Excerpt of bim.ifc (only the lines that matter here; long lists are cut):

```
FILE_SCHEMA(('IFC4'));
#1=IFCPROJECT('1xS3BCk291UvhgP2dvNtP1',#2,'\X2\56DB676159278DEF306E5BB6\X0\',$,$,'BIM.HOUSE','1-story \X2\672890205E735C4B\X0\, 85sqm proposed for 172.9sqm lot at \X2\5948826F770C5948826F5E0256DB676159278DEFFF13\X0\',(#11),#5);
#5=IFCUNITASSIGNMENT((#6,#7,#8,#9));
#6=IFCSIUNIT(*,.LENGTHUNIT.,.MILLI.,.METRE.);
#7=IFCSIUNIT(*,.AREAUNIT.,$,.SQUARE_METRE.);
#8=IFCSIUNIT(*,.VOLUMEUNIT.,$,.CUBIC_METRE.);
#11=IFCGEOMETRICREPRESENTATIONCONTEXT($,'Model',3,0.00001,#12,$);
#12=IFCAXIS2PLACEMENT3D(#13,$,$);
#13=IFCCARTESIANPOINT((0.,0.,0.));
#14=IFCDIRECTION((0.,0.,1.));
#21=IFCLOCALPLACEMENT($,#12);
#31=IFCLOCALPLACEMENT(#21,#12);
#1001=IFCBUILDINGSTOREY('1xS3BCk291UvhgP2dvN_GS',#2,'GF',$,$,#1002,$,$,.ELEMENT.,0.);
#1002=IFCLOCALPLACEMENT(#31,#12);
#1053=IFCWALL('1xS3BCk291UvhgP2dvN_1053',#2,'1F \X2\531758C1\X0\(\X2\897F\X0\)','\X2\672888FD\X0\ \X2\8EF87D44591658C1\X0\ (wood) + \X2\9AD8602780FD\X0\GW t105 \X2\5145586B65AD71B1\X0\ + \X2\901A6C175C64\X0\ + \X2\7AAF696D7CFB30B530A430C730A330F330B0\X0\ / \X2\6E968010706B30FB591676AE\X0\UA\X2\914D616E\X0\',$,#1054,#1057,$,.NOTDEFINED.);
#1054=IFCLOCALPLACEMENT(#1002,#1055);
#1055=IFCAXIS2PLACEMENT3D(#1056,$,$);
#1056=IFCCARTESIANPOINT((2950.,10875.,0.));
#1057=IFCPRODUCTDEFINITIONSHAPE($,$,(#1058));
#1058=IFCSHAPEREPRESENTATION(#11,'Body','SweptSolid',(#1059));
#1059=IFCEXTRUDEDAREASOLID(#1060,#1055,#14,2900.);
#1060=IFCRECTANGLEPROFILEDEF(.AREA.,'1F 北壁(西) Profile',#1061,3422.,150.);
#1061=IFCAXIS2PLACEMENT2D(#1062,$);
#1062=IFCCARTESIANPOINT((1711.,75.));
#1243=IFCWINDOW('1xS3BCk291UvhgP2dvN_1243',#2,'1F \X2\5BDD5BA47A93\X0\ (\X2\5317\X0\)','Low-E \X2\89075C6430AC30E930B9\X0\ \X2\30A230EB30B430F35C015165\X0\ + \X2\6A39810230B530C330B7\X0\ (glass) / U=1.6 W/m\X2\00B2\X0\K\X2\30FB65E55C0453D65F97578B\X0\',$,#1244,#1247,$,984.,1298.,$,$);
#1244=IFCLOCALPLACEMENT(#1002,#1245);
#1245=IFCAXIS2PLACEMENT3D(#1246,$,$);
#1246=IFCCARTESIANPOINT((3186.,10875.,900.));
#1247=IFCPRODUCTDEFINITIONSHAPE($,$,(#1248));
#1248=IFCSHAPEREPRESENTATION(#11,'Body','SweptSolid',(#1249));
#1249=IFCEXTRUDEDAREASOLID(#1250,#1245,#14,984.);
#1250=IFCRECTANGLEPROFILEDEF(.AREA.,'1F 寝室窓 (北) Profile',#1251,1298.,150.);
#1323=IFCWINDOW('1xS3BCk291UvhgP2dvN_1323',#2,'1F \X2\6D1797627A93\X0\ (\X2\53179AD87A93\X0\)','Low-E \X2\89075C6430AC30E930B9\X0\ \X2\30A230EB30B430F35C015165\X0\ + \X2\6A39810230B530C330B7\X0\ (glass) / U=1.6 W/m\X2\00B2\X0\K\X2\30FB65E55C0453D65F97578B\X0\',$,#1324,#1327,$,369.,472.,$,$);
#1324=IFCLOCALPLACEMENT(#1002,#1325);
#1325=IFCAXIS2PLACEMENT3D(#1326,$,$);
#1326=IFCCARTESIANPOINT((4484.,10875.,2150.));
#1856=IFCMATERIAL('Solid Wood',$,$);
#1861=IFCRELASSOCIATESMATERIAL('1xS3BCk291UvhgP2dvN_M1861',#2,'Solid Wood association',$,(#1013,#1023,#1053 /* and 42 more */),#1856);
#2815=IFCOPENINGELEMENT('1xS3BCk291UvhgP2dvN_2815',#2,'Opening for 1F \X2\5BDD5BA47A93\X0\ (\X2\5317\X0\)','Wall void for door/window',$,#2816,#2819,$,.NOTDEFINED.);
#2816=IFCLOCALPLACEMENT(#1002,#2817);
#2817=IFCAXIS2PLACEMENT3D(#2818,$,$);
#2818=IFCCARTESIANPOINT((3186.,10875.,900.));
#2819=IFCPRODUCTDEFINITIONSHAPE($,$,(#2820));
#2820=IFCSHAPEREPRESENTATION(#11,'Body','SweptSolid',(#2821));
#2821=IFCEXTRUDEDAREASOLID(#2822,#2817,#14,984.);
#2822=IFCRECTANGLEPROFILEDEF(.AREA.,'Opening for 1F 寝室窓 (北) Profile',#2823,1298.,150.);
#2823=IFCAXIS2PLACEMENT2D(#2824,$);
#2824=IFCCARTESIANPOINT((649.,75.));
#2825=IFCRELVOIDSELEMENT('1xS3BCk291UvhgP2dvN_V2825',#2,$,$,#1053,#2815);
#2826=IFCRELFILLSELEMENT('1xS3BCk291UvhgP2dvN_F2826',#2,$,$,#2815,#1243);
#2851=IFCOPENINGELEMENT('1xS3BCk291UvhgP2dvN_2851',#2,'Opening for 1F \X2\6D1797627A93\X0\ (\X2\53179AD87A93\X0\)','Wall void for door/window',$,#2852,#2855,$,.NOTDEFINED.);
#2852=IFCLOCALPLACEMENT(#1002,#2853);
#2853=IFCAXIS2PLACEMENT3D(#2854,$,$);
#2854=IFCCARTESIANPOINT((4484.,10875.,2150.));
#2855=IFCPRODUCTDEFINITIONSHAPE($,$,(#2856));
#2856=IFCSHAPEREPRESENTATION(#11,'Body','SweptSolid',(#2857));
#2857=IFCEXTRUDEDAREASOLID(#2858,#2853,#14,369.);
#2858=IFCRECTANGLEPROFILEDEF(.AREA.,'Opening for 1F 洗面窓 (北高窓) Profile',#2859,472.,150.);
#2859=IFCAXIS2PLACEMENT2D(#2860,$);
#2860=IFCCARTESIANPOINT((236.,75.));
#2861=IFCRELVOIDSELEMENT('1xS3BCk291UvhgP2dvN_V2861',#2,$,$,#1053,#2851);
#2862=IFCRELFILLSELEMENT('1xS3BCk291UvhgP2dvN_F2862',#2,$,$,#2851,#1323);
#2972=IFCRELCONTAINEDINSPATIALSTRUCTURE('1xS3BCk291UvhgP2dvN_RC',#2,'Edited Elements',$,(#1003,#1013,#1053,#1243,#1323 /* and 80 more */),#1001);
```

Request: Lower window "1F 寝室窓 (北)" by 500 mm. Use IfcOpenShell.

```python
import numpy as np
import ifcopenshell
import ifcopenshell.api.geometry
import ifcopenshell.util.placement
import ifcopenshell.util.unit

model = ifcopenshell.open("bim.ifc")
unit_scale = ifcopenshell.util.unit.calculate_unit_scale(model)

window = model.by_id(1243)
opening = window.FillsVoids[0].RelatingOpeningElement
dz = -500.0

shift = np.array([0.0, 0.0, dz])
# The window is not placed relative to its opening, so move both.
for product in (opening, window):
    matrix = ifcopenshell.util.placement.get_local_placement(product.ObjectPlacement)
    matrix[:3, 3] += shift
    ifcopenshell.api.geometry.edit_object_placement(model, product=product, matrix=matrix, is_si=False)

print(f"moved by {dz * unit_scale:+.3f} m")

model.write("bim_rev.ifc")
```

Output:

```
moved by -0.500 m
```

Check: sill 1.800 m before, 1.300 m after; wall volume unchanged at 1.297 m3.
